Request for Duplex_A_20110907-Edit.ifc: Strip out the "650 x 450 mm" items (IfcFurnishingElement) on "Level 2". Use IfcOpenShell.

First a look at what the model holds.

```python
import ifcopenshell
import ifcopenshell.util.element

model = ifcopenshell.open("Duplex_A_20110907-Edit.ifc")
print(model.schema)
storey = next(s for s in model.by_type("IfcBuildingStorey") if s.Name == "Level 2")
furniture = [e for e in ifcopenshell.util.element.get_decomposition(storey) if e.is_a("IfcFurnishingElement")]
seen = {}
for e in furniture:
    element_type = ifcopenshell.util.element.get_type(e)
    name = element_type.Name if element_type not in (None, e) else None
    seen[name] = seen.get(name, 0) + 1
for name, count in sorted(seen.items(), key=str):
    print(count, "x", name)
```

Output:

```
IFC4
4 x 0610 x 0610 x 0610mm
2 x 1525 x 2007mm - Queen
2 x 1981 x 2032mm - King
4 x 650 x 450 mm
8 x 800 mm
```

```python
import ifcopenshell
import ifcopenshell.api.root
import ifcopenshell.util.element

model = ifcopenshell.open("Duplex_A_20110907-Edit.ifc")

storey = next(s for s in model.by_type("IfcBuildingStorey") if s.Name == "Level 2")
furniture = [e for e in ifcopenshell.util.element.get_decomposition(storey) if e.is_a("IfcFurnishingElement")]
targets = [e for e in furniture if (t := ifcopenshell.util.element.get_type(e)) not in (None, e) and t.Name == "650 x 450 mm"]

for e in targets:
    ifcopenshell.api.root.remove_product(model, product=e)
print(len(targets), "removed")

model.write("Duplex_A_20110907-Edit-out.ifc")
```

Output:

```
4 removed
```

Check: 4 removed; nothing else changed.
